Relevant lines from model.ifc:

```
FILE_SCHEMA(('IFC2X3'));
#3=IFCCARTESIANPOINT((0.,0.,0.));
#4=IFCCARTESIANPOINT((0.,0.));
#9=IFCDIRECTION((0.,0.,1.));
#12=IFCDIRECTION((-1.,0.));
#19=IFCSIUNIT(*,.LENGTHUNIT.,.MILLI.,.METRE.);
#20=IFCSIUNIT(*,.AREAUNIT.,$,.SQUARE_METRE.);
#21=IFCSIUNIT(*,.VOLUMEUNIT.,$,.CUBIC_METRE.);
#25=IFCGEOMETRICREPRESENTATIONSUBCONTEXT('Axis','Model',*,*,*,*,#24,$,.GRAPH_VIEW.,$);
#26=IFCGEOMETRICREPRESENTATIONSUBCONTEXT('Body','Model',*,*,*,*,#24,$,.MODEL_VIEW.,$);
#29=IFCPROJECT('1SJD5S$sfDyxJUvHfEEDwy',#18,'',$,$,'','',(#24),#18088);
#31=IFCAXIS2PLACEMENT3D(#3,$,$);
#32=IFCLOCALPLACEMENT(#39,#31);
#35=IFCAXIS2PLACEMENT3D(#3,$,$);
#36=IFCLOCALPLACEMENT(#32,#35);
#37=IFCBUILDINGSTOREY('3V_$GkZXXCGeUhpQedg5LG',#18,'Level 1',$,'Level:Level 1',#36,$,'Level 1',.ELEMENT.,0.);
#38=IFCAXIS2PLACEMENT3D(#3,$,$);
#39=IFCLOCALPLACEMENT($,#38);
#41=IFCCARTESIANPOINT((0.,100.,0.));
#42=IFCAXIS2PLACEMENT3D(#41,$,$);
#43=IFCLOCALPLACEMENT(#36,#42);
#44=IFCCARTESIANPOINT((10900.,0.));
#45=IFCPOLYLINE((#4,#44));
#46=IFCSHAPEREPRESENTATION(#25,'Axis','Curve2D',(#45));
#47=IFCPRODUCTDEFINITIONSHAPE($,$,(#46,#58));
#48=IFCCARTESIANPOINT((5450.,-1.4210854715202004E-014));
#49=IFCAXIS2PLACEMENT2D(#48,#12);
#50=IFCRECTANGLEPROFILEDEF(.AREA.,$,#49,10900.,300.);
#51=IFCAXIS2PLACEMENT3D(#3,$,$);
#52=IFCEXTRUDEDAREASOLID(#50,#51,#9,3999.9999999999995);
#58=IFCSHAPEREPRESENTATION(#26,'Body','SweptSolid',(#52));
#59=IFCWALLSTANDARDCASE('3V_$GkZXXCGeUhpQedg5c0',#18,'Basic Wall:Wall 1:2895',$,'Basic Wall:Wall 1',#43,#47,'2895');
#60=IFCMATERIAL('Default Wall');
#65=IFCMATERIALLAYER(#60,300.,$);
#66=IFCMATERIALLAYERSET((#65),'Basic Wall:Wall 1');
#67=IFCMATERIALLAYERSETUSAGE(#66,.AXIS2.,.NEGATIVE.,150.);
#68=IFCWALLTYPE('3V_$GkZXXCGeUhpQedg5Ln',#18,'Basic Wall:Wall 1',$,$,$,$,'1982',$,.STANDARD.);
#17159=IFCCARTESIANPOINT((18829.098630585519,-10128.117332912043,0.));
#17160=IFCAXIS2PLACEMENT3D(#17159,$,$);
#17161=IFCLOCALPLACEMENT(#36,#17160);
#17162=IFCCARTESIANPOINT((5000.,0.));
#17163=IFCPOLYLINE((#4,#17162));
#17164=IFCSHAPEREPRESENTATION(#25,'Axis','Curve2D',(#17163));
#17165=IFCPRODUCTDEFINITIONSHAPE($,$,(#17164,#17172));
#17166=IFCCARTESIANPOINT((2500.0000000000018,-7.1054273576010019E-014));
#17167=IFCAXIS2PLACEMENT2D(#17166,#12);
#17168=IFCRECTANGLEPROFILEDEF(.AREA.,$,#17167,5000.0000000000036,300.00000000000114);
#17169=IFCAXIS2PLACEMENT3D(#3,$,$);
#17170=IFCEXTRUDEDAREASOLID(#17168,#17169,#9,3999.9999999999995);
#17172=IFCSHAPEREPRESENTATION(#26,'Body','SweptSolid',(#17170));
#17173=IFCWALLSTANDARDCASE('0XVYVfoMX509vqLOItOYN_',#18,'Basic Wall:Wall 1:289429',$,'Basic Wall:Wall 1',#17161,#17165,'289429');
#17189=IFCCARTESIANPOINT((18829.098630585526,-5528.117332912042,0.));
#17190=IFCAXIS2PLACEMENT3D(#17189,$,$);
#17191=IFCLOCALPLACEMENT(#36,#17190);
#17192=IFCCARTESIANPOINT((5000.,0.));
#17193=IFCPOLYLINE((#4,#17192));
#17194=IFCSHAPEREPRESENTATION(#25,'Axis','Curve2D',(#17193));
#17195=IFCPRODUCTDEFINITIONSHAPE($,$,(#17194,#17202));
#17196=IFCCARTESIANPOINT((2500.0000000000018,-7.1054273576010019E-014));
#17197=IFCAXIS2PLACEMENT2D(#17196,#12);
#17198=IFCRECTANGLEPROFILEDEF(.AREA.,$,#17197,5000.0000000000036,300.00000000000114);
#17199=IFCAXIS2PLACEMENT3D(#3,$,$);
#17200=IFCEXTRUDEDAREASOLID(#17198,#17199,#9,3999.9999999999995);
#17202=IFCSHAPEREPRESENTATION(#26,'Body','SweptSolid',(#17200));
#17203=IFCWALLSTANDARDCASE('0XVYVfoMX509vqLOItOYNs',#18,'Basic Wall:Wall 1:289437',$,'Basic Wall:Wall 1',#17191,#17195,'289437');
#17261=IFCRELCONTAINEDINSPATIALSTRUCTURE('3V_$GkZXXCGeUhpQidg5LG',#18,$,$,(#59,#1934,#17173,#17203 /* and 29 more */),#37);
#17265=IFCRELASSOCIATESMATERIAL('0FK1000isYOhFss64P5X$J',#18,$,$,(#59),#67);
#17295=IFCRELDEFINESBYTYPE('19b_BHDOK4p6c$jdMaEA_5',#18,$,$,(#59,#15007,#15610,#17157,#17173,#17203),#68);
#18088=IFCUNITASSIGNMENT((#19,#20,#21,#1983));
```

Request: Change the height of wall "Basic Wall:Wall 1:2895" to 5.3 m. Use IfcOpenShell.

```python
import ifcopenshell
import ifcopenshell.geom
import ifcopenshell.util.representation
import ifcopenshell.util.shape
import ifcopenshell.util.unit

model = ifcopenshell.open("model.ifc")
unit_scale = ifcopenshell.util.unit.calculate_unit_scale(model)
settings = ifcopenshell.geom.settings()


def volume(element):
    """Net volume in cubic metres, openings subtracted."""
    shape = ifcopenshell.geom.create_shape(settings, element)
    return ifcopenshell.util.shape.get_volume(shape.geometry)


wall = model.by_id(59)
before = volume(wall)

body = ifcopenshell.util.representation.get_representation(wall, "Model", "Body")
solid = body.Items[0]
old_height = solid.Depth
solid.Depth = 5.3 / unit_scale
after = volume(wall)

print(f"height {old_height:g} -> {solid.Depth:g}, volume {before:.3f} -> {after:.3f} m3")

model.write("model_rev.ifc")
```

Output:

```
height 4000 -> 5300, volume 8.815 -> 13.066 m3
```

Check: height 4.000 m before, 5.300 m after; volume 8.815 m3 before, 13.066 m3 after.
